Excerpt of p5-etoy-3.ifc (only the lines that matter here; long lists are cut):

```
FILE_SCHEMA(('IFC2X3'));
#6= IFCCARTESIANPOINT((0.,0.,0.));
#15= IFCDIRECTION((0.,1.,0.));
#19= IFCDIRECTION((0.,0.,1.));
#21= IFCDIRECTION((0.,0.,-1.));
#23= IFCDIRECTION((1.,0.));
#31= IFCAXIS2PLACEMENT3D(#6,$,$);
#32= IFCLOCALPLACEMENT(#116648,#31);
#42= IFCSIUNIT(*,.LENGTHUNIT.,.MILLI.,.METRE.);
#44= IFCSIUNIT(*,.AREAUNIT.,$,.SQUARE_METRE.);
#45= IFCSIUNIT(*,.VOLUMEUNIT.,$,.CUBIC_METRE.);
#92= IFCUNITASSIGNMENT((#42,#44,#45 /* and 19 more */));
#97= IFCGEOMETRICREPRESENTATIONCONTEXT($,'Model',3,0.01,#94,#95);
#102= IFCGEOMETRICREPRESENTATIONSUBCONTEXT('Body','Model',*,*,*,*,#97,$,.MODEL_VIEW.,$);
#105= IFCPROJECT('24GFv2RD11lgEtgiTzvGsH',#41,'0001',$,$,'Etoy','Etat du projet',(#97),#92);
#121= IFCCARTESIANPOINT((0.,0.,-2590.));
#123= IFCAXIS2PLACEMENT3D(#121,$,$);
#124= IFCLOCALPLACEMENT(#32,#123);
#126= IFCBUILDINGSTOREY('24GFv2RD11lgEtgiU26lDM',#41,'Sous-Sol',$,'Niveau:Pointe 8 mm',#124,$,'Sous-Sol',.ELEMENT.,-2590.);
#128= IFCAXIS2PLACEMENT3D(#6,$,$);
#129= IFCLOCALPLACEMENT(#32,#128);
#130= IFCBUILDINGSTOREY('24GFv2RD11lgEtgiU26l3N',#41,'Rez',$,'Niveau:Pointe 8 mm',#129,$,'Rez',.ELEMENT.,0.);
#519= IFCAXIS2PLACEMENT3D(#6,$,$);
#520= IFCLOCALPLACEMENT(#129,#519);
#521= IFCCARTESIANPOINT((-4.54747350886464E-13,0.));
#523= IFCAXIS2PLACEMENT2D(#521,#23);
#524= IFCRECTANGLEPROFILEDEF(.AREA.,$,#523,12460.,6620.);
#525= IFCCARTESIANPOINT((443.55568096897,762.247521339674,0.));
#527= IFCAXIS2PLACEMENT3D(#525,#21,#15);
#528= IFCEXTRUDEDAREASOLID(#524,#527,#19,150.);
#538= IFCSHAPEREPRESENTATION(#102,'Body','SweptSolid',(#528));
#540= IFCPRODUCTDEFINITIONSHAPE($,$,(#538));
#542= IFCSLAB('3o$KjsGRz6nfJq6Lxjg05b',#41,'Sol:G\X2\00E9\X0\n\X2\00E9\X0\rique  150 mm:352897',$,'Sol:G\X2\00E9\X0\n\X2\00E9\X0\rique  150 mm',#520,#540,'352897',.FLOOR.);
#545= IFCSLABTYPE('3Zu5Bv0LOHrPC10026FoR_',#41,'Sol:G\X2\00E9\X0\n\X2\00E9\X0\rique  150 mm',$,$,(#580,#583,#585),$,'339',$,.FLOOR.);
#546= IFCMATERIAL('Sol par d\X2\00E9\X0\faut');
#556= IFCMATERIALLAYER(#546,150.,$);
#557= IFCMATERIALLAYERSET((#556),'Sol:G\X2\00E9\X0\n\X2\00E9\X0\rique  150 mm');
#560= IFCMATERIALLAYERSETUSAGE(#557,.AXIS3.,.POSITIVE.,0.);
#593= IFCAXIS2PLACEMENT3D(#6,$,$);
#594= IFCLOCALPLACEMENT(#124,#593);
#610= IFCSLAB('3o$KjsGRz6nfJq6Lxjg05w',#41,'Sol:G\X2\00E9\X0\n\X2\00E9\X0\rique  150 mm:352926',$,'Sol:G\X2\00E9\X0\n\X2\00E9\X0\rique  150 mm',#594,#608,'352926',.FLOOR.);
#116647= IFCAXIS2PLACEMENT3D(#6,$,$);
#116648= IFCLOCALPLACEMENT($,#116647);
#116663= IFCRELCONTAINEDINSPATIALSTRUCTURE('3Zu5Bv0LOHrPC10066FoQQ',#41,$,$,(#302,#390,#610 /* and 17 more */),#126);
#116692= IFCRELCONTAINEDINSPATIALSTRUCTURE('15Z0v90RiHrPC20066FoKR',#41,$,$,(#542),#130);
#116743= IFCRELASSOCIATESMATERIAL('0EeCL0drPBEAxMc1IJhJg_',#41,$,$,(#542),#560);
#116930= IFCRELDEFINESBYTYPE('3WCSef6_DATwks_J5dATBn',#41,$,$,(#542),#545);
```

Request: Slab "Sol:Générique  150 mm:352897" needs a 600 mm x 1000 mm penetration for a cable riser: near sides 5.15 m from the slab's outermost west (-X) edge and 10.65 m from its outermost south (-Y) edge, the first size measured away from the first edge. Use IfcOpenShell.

```python
import numpy as np
import ifcopenshell
import ifcopenshell.api.feature
import ifcopenshell.api.geometry
import ifcopenshell.api.root
import ifcopenshell.geom
import ifcopenshell.util.placement
import ifcopenshell.util.representation
import ifcopenshell.util.shape
import ifcopenshell.util.unit

model = ifcopenshell.open("p5-etoy-3.ifc")
unit_scale = ifcopenshell.util.unit.calculate_unit_scale(model)
settings = ifcopenshell.geom.settings()


def volume(element):
    """Net volume in cubic metres, openings subtracted."""
    shape = ifcopenshell.geom.create_shape(settings, element)
    return ifcopenshell.util.shape.get_volume(shape.geometry)


slab = model.by_guid("3o$KjsGRz6nfJq6Lxjg05b")
before = volume(slab)

# Extent in the slab's own axes, in metres. The edges named are its -X and -Y sides.
slab_shape = ifcopenshell.geom.create_shape(settings, slab)
vertices = ifcopenshell.util.shape.get_vertices(slab_shape.geometry)
x_min, y_min, bottom = vertices.min(axis=0)
top = vertices[:, 2].max()

opening = ifcopenshell.api.root.create_entity(model, ifc_class="IfcOpeningElement", name="Cable riser opening")
context = ifcopenshell.util.representation.get_context(model, "Model", "Body", "MODEL_VIEW")
width, depth = 0.6, 1
outline = [(0.0, 0.0), (width, 0.0), (width, depth), (0.0, depth), (0.0, 0.0)]
# Overshoot both faces by 50 mm so the cut is clean.
shape = ifcopenshell.api.geometry.add_slab_representation(
    model, context=context, depth=top - bottom + 0.1, polyline=outline
)
ifcopenshell.api.geometry.assign_representation(model, product=opening, representation=shape)

matrix = ifcopenshell.util.placement.get_local_placement(slab.ObjectPlacement)
matrix[:, 3] = matrix @ np.append(np.array([x_min + 5.15, y_min + 10.65, bottom - 0.05]) / unit_scale, 1.0)
ifcopenshell.api.geometry.edit_object_placement(model, product=opening, matrix=matrix, is_si=False)
ifcopenshell.api.feature.add_feature(model, feature=opening, element=slab)

after = volume(slab)

print(f"slab volume {before:.3f} -> {after:.3f} m3")

model.write("p5-etoy-3_edited.ifc")
```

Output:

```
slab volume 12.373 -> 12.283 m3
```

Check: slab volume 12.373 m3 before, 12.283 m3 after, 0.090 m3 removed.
